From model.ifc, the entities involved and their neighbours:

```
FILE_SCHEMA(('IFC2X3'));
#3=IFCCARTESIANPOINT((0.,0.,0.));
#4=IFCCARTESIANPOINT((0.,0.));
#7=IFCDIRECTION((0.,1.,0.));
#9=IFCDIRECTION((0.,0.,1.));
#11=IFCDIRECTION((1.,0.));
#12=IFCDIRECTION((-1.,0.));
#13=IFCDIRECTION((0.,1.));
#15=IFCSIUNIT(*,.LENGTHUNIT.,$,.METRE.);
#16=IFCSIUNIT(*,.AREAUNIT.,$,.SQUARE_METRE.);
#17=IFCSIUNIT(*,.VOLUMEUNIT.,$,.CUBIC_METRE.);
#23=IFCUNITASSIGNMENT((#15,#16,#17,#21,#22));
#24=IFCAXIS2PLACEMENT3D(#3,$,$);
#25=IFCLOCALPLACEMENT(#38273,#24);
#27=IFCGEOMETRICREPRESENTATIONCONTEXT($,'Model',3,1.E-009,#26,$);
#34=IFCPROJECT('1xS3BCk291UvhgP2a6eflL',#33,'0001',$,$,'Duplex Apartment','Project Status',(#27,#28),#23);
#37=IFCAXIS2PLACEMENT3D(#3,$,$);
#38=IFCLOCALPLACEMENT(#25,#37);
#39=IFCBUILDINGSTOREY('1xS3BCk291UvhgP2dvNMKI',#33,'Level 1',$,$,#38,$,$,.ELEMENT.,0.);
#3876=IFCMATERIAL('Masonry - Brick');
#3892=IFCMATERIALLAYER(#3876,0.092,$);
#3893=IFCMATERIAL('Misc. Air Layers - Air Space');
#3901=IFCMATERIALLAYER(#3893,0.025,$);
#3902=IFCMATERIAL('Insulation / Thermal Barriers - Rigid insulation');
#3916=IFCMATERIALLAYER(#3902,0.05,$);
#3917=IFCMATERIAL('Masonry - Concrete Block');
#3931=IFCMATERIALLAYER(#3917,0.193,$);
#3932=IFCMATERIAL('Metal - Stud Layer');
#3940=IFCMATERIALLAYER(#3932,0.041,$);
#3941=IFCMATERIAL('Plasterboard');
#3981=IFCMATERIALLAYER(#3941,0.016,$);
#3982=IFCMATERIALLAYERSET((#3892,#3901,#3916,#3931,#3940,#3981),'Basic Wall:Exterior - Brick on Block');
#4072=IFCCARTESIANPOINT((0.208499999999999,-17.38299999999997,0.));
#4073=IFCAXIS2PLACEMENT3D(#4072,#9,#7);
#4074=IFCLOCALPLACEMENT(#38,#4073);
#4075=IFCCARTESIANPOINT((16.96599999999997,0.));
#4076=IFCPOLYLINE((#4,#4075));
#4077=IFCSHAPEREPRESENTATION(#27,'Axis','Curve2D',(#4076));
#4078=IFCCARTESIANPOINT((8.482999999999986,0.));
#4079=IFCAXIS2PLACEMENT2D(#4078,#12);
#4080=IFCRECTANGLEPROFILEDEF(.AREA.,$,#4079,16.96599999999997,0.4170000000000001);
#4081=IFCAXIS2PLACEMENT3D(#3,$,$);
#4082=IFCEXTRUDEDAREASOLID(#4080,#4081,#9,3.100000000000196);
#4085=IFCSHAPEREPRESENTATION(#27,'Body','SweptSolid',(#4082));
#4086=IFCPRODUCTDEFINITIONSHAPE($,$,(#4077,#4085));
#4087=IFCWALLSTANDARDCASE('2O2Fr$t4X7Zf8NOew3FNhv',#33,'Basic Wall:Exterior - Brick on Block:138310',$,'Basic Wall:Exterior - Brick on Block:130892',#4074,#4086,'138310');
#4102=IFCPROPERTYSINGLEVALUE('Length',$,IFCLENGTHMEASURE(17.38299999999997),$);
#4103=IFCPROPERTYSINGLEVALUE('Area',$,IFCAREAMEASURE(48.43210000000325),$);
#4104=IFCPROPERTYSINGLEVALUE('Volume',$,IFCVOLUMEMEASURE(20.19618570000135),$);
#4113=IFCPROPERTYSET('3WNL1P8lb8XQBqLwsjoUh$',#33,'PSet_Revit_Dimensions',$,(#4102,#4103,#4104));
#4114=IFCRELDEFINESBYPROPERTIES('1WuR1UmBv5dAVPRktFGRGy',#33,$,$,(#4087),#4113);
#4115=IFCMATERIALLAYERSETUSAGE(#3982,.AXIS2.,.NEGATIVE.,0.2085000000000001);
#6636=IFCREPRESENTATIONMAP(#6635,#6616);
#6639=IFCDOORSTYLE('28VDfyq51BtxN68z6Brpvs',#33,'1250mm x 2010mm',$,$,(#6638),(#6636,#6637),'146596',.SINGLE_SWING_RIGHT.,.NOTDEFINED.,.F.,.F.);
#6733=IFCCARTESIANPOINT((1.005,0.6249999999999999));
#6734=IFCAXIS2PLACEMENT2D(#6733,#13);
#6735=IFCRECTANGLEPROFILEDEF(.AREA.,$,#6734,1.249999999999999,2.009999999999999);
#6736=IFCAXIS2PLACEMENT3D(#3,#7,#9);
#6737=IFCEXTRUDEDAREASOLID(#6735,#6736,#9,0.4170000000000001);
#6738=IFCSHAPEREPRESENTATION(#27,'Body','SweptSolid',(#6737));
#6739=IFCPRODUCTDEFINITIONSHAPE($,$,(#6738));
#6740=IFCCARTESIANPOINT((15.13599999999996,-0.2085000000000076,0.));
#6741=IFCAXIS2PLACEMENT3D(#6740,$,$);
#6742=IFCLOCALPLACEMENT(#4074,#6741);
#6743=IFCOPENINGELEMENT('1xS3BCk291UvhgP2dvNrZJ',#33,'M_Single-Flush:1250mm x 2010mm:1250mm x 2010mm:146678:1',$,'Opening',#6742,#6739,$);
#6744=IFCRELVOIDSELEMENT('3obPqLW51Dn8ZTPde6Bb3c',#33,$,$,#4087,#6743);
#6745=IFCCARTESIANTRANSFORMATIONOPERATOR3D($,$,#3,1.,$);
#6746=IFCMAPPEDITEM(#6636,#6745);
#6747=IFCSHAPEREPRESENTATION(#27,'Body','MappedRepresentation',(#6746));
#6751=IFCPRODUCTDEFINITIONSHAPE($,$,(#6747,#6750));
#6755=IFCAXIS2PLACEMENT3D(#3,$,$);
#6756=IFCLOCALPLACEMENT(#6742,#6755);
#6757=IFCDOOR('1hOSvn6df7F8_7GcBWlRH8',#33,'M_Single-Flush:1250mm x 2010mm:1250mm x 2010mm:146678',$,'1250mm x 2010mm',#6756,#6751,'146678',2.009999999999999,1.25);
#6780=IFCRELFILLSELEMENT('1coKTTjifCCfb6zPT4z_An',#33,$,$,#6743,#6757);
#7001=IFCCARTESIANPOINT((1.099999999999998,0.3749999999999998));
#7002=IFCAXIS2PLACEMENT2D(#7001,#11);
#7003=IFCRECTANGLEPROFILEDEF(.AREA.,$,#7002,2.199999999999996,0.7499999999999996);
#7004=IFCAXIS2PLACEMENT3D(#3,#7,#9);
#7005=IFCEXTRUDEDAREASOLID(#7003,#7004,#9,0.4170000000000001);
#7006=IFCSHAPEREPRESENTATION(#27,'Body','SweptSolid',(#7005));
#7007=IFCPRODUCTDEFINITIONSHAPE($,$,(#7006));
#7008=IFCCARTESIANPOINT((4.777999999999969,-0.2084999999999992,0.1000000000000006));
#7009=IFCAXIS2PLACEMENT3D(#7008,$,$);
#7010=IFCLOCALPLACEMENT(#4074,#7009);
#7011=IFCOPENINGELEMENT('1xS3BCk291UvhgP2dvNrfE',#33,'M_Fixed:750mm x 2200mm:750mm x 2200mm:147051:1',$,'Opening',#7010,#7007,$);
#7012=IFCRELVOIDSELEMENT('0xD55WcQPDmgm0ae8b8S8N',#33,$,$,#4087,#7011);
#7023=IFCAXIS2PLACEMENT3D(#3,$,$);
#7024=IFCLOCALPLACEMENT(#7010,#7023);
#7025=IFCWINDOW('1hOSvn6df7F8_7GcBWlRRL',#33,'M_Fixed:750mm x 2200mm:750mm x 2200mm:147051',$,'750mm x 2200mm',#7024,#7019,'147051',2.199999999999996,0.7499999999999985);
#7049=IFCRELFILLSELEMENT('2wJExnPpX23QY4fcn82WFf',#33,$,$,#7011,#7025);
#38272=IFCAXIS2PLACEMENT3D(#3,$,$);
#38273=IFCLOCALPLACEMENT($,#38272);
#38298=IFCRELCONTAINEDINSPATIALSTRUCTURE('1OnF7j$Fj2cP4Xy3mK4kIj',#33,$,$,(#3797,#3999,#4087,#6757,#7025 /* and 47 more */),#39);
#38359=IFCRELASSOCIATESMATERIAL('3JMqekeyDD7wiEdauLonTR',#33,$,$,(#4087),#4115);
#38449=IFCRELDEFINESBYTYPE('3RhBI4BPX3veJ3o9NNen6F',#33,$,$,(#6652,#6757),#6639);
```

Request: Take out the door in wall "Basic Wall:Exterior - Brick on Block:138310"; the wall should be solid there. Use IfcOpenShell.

```python
import ifcopenshell
import ifcopenshell.api.feature
import ifcopenshell.api.pset
import ifcopenshell.api.root
import ifcopenshell.geom
import ifcopenshell.util.element
import ifcopenshell.util.shape
import ifcopenshell.util.unit

model = ifcopenshell.open("model.ifc")
area_scale = ifcopenshell.util.unit.calculate_unit_scale(model, "AREAUNIT")
volume_scale = ifcopenshell.util.unit.calculate_unit_scale(model, "VOLUMEUNIT")
settings = ifcopenshell.geom.settings()


def volume(element):
    """Net volume in cubic metres, openings subtracted."""
    shape = ifcopenshell.geom.create_shape(settings, element)
    return ifcopenshell.util.shape.get_volume(shape.geometry)


door = model.by_id(6757)
opening = door.FillsVoids[0].RelatingOpeningElement
wall = opening.VoidsElements[0].RelatingBuildingElement
before = volume(wall)

ifcopenshell.api.root.remove_product(model, product=door)
ifcopenshell.api.feature.remove_feature(model, feature=opening)

after = volume(wall)
thickness = 0.417  # wall thickness in metres

# Update the wall's stored quantities.
pset = model.by_id(ifcopenshell.util.element.get_pset(wall, "PSet_Revit_Dimensions", should_inherit=False)["id"])
ifcopenshell.api.pset.edit_pset(model, pset=pset, properties={
    "Area": model.create_entity("IfcAreaMeasure", after / thickness / area_scale),
    "Volume": model.create_entity("IfcVolumeMeasure", after / volume_scale),
})

print(f"wall volume {before:.3f} -> {after:.3f} m3")

model.write("model_edited.ifc")
```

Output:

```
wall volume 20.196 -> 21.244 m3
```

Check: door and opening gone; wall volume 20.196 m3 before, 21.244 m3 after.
